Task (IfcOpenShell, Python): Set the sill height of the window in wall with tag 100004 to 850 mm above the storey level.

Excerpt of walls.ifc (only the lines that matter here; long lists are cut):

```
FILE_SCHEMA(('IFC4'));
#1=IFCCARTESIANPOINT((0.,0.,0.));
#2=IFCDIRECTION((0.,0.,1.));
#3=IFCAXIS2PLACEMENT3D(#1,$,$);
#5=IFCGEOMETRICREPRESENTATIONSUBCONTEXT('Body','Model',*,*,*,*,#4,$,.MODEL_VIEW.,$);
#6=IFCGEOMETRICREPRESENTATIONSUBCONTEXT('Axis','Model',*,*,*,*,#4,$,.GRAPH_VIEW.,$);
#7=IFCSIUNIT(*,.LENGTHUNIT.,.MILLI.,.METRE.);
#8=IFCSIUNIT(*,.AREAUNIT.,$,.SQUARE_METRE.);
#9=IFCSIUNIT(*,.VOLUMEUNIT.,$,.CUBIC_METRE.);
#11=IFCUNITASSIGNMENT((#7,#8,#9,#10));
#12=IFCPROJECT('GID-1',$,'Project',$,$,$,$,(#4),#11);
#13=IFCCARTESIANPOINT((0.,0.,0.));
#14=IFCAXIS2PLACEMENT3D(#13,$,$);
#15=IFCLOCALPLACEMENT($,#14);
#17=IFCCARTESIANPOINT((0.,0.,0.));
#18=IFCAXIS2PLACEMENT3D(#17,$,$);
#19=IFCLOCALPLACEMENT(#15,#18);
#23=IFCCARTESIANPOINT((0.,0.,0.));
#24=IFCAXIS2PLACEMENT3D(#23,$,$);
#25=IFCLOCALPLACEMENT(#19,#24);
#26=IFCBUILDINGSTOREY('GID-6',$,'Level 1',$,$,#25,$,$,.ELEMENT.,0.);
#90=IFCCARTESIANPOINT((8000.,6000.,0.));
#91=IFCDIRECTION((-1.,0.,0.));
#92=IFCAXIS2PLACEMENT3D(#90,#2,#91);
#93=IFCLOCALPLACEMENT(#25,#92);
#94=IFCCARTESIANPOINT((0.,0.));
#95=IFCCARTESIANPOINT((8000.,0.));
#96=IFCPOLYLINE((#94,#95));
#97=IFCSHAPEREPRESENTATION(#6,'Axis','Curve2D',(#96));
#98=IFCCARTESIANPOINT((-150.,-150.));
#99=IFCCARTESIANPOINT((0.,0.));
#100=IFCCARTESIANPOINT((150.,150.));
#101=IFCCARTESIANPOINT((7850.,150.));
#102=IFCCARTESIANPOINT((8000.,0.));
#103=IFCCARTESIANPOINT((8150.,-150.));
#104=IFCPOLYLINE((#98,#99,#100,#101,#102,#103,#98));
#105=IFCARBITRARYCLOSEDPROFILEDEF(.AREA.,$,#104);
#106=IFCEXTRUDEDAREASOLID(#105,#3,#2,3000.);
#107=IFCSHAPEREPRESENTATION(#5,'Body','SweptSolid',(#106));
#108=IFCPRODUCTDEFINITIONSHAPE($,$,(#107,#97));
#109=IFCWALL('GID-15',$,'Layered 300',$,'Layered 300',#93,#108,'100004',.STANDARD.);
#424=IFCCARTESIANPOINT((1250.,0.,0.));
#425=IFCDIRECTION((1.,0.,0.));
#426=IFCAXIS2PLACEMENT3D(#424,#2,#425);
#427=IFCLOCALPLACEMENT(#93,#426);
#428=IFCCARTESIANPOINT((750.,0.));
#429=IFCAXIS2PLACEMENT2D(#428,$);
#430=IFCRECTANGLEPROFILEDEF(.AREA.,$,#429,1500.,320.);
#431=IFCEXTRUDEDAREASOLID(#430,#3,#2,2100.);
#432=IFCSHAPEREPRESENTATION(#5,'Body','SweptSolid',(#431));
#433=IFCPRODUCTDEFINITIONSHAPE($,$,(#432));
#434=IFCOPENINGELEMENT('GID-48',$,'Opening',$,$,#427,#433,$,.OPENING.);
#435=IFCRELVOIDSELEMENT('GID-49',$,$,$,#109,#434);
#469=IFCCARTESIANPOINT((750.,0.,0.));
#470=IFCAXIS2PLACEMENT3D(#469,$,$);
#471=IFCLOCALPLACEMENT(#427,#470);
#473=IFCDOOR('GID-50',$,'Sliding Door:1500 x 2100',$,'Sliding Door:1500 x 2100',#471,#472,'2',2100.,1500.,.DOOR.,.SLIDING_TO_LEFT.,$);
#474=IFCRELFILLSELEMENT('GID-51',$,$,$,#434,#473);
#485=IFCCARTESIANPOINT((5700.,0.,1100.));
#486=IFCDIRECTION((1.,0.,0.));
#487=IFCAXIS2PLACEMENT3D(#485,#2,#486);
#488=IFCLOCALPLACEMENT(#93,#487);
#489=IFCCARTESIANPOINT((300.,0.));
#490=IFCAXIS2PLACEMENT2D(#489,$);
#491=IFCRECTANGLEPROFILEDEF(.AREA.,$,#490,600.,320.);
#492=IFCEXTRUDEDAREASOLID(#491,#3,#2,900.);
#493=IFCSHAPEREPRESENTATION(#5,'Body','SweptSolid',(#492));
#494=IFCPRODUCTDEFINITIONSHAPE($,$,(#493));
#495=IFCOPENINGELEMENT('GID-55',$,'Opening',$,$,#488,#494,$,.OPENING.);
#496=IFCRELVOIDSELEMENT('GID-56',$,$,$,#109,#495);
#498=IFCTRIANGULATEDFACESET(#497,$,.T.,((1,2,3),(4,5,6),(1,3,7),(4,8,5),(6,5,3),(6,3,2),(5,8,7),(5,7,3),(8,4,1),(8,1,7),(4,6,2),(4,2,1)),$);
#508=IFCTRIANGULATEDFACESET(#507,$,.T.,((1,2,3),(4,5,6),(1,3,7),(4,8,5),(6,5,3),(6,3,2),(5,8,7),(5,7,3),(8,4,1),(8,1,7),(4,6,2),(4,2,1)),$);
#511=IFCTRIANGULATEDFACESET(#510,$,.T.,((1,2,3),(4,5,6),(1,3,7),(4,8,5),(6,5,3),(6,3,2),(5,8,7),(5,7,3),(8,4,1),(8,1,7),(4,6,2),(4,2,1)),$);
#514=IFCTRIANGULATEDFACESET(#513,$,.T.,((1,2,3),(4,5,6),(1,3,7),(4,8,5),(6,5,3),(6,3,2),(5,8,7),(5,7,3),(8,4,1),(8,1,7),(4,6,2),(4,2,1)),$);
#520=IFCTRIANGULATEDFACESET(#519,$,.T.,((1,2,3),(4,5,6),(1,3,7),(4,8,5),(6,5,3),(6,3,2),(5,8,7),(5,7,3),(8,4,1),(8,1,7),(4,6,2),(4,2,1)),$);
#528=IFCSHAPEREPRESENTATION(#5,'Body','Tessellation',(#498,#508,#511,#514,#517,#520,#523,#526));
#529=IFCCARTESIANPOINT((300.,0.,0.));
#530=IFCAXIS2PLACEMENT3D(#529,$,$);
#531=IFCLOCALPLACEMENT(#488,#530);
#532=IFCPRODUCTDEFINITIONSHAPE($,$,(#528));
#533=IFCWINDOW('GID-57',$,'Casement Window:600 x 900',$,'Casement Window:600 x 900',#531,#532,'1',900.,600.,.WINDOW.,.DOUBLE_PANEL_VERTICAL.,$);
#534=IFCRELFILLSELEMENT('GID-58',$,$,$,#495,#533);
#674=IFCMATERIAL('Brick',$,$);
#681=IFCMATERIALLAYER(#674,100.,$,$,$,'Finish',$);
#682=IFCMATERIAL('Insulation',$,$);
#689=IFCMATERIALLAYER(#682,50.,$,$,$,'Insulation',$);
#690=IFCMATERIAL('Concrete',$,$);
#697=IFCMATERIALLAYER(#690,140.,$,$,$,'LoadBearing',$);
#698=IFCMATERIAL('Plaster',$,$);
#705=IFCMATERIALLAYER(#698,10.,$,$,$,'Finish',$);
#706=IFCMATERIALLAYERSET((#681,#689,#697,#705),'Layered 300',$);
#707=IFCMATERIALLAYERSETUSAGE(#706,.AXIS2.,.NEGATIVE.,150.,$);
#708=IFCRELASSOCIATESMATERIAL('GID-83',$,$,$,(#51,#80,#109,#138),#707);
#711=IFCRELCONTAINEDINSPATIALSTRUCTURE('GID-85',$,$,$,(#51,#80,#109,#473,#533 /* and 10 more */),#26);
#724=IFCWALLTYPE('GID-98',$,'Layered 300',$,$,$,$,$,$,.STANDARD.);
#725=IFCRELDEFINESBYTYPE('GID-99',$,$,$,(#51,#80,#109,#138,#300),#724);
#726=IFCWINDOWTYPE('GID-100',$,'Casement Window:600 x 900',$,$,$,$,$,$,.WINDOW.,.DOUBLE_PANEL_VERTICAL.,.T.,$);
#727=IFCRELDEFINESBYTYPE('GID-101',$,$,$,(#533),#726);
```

```python
import numpy as np
import ifcopenshell
import ifcopenshell.api.geometry
import ifcopenshell.geom
import ifcopenshell.util.element
import ifcopenshell.util.placement
import ifcopenshell.util.shape
import ifcopenshell.util.unit

model = ifcopenshell.open("walls.ifc")
unit_scale = ifcopenshell.util.unit.calculate_unit_scale(model)

window = model.by_guid("GID-57")
opening = window.FillsVoids[0].RelatingOpeningElement
storey = ifcopenshell.util.element.get_container(window, ifc_class="IfcBuildingStorey")
level = ifcopenshell.util.placement.get_local_placement(storey.ObjectPlacement)[2, 3]

# The opening's origin need not be at the sill, so measure its lowest point.
shape = ifcopenshell.geom.create_shape(ifcopenshell.geom.settings(), opening)
bottom = ifcopenshell.util.shape.get_shape_bottom_elevation(shape, shape.geometry) / unit_scale
dz = level + 0.85 / unit_scale - bottom

shift = np.array([0.0, 0.0, dz])
# The window is placed relative to its opening, so it follows when the opening moves.
matrix = ifcopenshell.util.placement.get_local_placement(opening.ObjectPlacement)
matrix[:3, 3] += shift
ifcopenshell.api.geometry.edit_object_placement(
    model, product=opening, matrix=matrix, is_si=False, should_transform_children=True
)

print(f"moved by {dz * unit_scale:+.3f} m")

model.write("walls_v2.ifc")
```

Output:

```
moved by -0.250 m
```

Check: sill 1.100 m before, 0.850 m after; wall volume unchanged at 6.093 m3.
